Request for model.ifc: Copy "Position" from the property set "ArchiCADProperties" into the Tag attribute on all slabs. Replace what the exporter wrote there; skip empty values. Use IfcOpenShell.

First a look at what the model holds.

```python
import ifcopenshell
import ifcopenshell.util.element

model = ifcopenshell.open("model.ifc")
print(model.schema)
slabs = model.by_type("IfcSlab")
print(len(slabs), "slabs")
for e in slabs[:8]:
    source = ifcopenshell.util.element.get_pset(e, "ArchiCADProperties", "Position")
    target = e.Tag
    print(e.id(), repr(source), repr(target), sep=" | ")
```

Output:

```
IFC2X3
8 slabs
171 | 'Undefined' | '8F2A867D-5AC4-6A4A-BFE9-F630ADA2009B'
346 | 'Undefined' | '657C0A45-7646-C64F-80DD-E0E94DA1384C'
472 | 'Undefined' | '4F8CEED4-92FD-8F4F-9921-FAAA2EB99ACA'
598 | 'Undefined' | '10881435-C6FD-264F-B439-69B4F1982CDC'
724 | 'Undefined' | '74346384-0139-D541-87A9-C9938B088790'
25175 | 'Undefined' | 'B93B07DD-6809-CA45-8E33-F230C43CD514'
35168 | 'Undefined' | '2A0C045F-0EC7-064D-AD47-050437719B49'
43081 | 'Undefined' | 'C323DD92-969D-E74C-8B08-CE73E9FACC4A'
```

```python
import ifcopenshell
import ifcopenshell.util.element

model = ifcopenshell.open("model.ifc")

count = 0
for e in model.by_type("IfcSlab"):
    value = ifcopenshell.util.element.get_pset(e, "ArchiCADProperties", "Position")
    current = e.Tag
    if not value or not value.strip() or current == value:
        continue
    e.Tag = value
    count += 1

print(count, "slabs updated")

model.write("model_updated.ifc")
```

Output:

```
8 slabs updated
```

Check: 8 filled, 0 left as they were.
